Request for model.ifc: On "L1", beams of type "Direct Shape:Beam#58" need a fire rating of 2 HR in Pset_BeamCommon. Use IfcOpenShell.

First a look at what the model holds.

```python
import ifcopenshell
import ifcopenshell.util.element

model = ifcopenshell.open("model.ifc")
print(model.schema)
storey = next(s for s in model.by_type("IfcBuildingStorey") if s.Name == "L1")
beams = [e for e in ifcopenshell.util.element.get_decomposition(storey) if e.is_a("IfcBeam")]
seen = {}
for e in beams:
    element_type = ifcopenshell.util.element.get_type(e)
    key = (element_type.Name if element_type != e and element_type else None, ifcopenshell.util.element.get_pset(e, "Pset_BeamCommon", "FireRating"))
    seen[key] = seen.get(key, 0) + 1
for (name, value), count in sorted(seen.items(), key=str):
    print(count, "x", name, "|", value)
```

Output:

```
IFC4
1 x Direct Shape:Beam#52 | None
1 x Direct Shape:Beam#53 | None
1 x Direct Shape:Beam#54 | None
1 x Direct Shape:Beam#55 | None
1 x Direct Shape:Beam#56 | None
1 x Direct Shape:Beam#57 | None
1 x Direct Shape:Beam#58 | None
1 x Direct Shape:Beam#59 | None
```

```python
import ifcopenshell
import ifcopenshell.api.pset
import ifcopenshell.util.element

model = ifcopenshell.open("model.ifc")

storey = next(s for s in model.by_type("IfcBuildingStorey") if s.Name == "L1")
beams = [e for e in ifcopenshell.util.element.get_decomposition(storey) if e.is_a("IfcBeam")]

count = 0
for e in beams:
    element_type = ifcopenshell.util.element.get_type(e)
    if element_type in (None, e) or element_type.Name != "Direct Shape:Beam#58":
        continue
    # add_pset returns the element's existing set when there is one.
    pset = ifcopenshell.api.pset.add_pset(model, product=e, name="Pset_BeamCommon")
    ifcopenshell.api.pset.edit_pset(model, pset=pset, properties={"FireRating": "2 HR"})
    count += 1

print(count, "beams updated")

model.write("model-out.ifc")
```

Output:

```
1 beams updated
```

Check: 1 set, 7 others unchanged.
